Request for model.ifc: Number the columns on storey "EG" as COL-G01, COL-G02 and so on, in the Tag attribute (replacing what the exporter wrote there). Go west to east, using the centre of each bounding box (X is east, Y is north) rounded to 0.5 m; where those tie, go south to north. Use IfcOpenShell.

First a look at what the model holds.

```python
import ifcopenshell
import ifcopenshell.util.element
import ifcopenshell.util.placement

model = ifcopenshell.open("model.ifc")
print(model.schema)
storey = next(s for s in model.by_type("IfcBuildingStorey") if s.Name == "EG")
columns = [e for e in ifcopenshell.util.element.get_decomposition(storey) if e.is_a("IfcColumn")]
for e in sorted(columns, key=lambda e: e.id()):
    origin = ifcopenshell.util.placement.get_local_placement(e.ObjectPlacement)[:3, 3]
    print(e.id(), e.Tag, e.Name, origin.round(2) + 0.0, sep=" | ")
```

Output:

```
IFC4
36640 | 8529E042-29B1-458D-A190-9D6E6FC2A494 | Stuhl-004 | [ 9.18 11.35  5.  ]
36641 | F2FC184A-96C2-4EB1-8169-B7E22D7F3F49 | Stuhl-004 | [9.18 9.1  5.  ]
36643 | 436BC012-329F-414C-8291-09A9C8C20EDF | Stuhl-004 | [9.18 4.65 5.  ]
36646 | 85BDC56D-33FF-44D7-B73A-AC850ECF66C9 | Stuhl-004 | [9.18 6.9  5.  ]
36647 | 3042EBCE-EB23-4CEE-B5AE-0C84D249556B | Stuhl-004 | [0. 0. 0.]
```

```python
import ifcopenshell
import ifcopenshell.geom
import ifcopenshell.util.element
import ifcopenshell.util.shape

model = ifcopenshell.open("model.ifc")
settings = ifcopenshell.geom.settings()
settings.set("use-world-coords", True)


def centre(element):
    shape = ifcopenshell.geom.create_shape(settings, element)
    return ifcopenshell.util.shape.get_bbox_centroid(shape.geometry)


storey = next(s for s in model.by_type("IfcBuildingStorey") if s.Name == "EG")
columns = [e for e in ifcopenshell.util.element.get_decomposition(storey) if e.is_a("IfcColumn")]

# Insertion points can sit at a corner or the storey origin, so sort by the geometry (in metres).
centres = {e: centre(e) for e in columns}
columns.sort(key=lambda e: (round(centres[e][0] / 0.5), centres[e][1]))

for i, e in enumerate(columns, start=1):
    number = f"COL-G{i:02d}"
    e.Tag = number
    print(e.id(), number)

model.write("model_rev.ifc")
```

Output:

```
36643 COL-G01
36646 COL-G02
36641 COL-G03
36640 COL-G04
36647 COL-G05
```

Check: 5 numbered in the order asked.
